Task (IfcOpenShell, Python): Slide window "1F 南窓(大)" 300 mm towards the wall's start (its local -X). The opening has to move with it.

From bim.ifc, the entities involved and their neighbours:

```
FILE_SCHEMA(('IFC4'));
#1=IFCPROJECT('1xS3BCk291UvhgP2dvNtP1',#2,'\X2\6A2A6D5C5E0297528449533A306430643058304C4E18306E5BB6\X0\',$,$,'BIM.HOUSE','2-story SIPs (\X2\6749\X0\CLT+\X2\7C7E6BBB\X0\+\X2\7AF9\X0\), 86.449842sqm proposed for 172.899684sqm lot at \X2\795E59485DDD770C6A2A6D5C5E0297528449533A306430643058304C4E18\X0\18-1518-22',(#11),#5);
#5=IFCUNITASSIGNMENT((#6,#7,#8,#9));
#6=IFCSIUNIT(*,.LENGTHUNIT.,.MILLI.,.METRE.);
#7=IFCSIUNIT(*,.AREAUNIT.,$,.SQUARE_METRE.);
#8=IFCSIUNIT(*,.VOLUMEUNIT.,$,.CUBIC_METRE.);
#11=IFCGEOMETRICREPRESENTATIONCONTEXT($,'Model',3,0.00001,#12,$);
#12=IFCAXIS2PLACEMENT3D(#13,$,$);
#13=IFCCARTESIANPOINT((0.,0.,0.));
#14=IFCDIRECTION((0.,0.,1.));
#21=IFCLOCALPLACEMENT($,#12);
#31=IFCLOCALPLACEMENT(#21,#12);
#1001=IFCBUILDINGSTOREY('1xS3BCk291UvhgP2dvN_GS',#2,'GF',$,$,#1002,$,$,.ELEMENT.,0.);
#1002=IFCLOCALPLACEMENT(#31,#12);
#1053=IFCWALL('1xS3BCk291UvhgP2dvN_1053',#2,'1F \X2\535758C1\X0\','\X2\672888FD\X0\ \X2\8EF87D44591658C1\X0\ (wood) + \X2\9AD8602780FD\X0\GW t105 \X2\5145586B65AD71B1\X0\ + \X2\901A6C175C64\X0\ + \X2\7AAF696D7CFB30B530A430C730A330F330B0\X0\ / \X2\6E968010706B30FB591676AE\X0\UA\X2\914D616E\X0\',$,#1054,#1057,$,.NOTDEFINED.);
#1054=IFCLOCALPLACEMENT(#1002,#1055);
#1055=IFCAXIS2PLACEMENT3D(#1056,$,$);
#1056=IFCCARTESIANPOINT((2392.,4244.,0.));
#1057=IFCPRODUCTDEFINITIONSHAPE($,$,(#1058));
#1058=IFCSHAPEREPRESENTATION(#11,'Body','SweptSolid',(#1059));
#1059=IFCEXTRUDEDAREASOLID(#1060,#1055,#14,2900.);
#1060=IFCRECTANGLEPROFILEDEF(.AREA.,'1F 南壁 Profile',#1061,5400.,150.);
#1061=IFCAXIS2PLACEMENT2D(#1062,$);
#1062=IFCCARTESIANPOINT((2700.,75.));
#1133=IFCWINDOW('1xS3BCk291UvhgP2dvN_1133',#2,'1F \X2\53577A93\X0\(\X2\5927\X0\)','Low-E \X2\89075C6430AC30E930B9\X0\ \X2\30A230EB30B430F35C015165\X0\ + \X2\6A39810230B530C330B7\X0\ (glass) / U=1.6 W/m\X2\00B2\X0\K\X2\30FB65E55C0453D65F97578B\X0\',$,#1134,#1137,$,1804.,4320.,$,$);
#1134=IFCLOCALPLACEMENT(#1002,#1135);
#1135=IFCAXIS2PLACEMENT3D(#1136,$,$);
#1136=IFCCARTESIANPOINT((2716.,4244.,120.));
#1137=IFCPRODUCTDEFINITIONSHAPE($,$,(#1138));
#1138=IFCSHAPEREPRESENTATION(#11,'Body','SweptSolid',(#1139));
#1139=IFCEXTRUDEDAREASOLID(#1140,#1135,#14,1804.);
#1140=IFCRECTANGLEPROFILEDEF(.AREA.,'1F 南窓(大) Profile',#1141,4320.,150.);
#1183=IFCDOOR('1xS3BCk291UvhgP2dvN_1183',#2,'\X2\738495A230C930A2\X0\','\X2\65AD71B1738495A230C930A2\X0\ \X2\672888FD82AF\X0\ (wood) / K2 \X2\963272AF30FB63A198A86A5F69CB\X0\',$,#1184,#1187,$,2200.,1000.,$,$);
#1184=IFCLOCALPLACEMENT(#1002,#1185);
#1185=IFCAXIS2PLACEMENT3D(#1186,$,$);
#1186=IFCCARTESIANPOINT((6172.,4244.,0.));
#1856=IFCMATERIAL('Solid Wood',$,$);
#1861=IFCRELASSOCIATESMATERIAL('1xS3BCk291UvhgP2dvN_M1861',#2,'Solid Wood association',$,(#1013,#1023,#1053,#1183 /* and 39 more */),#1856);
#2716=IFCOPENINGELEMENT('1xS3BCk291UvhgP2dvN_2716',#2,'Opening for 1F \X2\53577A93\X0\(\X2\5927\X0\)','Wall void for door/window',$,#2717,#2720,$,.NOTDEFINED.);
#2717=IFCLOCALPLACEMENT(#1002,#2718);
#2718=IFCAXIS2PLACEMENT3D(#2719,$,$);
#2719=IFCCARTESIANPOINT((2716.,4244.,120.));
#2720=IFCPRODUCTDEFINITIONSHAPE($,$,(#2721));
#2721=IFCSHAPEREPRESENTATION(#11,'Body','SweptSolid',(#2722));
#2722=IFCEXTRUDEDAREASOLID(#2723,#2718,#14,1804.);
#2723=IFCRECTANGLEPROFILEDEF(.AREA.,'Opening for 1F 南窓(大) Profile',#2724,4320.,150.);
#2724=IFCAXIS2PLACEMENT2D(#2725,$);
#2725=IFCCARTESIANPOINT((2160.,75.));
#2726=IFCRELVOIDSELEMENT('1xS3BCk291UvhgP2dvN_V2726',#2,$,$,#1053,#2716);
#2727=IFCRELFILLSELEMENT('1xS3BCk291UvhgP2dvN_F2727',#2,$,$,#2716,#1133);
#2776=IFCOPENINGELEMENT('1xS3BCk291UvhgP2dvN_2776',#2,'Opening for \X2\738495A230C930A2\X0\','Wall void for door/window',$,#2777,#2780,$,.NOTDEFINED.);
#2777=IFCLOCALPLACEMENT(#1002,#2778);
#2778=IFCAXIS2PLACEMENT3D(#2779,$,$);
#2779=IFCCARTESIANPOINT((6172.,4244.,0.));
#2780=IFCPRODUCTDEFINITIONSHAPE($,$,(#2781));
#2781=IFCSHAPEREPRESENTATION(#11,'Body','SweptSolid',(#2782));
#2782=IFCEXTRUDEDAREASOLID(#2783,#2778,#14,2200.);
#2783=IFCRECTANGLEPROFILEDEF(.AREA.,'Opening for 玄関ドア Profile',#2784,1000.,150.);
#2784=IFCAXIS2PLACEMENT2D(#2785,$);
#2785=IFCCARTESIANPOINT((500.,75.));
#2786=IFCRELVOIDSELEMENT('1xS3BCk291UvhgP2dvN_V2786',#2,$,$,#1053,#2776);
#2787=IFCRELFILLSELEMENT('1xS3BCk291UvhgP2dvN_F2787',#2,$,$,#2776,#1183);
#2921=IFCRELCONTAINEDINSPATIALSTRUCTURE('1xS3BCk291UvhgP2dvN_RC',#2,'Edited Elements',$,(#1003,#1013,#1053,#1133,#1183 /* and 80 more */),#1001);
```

```python
import ifcopenshell
import ifcopenshell.api.geometry
import ifcopenshell.util.placement

model = ifcopenshell.open("bim.ifc")

window = model.by_guid("1xS3BCk291UvhgP2dvN_1133")
opening = window.FillsVoids[0].RelatingOpeningElement
wall = opening.VoidsElements[0].RelatingBuildingElement

wall_matrix = ifcopenshell.util.placement.get_local_placement(wall.ObjectPlacement)
shift = wall_matrix[:3, 0] * -300.0
before = ifcopenshell.util.placement.get_local_placement(window.ObjectPlacement)[:3, 3].copy()

# The window is not placed relative to its opening, so move both.
for product in (opening, window):
    matrix = ifcopenshell.util.placement.get_local_placement(product.ObjectPlacement)
    matrix[:3, 3] += shift
    ifcopenshell.api.geometry.edit_object_placement(model, product=product, matrix=matrix, is_si=False)

after = ifcopenshell.util.placement.get_local_placement(window.ObjectPlacement)[:3, 3]
print("window moved by", (after - before).round(3) + 0.0)

model.write("bim-out.ifc")
```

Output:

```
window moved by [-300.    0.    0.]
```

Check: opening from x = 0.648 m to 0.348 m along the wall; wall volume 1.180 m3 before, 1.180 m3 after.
